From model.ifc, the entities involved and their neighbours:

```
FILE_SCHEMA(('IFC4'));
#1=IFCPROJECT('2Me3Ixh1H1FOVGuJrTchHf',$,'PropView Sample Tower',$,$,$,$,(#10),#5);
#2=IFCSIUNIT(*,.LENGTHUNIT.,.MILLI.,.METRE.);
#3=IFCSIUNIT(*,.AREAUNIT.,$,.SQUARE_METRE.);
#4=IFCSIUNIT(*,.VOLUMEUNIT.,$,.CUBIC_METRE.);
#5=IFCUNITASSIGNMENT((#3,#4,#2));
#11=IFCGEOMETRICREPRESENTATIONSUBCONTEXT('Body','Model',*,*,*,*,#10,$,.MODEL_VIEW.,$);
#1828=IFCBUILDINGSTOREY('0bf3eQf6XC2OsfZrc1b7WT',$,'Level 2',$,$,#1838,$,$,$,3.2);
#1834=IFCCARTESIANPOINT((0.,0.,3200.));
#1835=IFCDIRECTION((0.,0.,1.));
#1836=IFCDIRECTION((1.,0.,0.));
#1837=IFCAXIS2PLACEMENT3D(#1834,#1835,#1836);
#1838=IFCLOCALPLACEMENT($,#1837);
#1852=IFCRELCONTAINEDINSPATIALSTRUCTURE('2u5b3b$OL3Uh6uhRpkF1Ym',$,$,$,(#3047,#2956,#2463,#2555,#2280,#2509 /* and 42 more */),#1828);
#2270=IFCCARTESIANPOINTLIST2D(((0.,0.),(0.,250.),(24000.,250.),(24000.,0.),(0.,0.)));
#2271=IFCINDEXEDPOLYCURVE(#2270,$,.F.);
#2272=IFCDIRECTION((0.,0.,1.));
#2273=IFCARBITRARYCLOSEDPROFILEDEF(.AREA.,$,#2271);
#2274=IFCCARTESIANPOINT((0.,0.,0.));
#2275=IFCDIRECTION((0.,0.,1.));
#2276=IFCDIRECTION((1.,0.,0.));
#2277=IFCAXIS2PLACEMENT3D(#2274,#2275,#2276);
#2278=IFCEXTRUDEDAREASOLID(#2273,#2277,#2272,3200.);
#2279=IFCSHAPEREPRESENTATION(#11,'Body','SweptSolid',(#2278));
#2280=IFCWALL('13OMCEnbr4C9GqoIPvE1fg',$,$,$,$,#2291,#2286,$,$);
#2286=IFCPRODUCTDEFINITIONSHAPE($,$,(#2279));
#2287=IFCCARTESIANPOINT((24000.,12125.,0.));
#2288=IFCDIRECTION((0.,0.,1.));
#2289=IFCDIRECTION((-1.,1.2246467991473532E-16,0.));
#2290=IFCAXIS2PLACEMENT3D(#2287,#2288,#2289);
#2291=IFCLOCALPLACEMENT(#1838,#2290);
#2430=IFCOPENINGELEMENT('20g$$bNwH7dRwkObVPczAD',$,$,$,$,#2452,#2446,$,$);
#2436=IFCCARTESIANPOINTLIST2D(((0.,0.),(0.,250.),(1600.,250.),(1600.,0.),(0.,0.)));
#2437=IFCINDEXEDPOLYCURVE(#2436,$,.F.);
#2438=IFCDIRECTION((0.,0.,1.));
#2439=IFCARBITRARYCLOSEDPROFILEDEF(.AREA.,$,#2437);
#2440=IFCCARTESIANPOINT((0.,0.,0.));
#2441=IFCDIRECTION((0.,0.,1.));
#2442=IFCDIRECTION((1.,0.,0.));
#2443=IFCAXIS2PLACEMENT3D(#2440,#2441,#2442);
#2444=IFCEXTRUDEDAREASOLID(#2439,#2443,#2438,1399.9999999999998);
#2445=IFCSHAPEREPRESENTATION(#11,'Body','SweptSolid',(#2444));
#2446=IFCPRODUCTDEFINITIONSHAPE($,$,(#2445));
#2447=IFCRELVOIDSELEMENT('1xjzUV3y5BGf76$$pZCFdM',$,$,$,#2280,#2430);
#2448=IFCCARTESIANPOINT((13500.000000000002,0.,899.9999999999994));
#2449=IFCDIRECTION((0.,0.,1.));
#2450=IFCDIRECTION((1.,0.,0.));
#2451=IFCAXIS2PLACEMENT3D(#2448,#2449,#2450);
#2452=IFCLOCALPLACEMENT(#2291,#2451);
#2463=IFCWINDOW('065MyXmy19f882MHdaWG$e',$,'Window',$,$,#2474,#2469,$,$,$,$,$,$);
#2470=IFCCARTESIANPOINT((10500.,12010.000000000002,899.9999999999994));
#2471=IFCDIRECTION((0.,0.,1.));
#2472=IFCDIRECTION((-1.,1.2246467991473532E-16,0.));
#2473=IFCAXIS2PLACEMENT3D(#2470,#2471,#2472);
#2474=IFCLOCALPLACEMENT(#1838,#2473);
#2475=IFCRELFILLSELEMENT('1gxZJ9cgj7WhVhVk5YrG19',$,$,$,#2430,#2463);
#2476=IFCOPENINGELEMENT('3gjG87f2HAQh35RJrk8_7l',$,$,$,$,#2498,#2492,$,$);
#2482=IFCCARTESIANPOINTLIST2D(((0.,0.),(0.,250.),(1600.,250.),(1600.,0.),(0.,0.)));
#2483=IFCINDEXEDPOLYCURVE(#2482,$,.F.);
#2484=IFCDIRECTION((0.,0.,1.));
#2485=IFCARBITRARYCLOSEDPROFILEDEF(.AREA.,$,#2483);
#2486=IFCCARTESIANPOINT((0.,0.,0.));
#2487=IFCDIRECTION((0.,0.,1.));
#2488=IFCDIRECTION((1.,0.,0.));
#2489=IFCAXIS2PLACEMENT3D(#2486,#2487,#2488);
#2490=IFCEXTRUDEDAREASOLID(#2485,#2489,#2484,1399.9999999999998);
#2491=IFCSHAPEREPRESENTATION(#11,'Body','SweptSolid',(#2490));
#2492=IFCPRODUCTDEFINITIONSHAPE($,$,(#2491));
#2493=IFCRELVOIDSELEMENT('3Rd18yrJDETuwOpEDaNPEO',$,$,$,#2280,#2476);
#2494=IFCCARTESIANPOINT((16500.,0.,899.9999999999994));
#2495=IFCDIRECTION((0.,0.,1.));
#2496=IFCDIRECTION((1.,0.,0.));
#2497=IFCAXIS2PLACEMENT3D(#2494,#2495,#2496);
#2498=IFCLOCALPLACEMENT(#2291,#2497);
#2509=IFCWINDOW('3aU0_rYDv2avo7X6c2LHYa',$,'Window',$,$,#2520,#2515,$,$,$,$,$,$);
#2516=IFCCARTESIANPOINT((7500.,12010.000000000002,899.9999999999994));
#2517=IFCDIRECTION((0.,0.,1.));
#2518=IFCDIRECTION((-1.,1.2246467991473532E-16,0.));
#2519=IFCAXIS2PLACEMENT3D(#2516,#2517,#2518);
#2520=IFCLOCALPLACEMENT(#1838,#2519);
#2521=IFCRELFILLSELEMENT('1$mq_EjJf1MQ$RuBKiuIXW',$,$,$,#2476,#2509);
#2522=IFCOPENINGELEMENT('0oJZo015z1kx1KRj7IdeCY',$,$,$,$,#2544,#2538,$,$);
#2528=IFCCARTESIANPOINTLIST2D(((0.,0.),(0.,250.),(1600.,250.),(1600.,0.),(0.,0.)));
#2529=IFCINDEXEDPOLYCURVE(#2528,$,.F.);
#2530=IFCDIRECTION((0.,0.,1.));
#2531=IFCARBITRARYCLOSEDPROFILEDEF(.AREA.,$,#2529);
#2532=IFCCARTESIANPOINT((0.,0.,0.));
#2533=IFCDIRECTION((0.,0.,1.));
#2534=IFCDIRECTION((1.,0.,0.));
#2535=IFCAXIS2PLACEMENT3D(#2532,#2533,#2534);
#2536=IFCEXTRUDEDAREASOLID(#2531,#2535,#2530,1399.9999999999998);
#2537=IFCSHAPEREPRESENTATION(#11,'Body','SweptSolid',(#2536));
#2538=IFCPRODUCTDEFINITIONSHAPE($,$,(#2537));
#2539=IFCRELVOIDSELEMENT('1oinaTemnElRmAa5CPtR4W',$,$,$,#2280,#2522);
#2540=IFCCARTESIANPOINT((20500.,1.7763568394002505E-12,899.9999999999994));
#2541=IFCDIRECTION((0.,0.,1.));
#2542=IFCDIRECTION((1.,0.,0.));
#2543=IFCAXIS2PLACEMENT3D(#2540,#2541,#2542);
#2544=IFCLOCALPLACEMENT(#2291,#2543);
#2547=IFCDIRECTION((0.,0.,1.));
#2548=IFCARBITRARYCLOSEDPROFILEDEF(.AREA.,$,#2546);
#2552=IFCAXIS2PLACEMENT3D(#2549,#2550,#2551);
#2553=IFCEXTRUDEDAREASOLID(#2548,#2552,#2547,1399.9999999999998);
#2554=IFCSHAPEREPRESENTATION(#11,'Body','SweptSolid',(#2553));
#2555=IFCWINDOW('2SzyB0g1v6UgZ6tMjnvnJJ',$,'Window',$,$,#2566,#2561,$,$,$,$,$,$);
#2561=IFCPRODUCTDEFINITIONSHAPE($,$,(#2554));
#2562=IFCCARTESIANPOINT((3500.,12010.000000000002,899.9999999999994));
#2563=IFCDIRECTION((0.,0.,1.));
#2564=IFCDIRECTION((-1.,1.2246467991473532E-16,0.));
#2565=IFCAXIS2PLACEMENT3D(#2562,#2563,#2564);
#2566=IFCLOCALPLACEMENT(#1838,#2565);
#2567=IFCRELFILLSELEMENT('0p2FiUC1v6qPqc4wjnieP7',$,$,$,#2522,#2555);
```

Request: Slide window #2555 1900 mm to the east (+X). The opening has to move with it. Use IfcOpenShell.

```python
import ifcopenshell
import ifcopenshell.api.geometry
import ifcopenshell.util.placement
import ifcopenshell.util.unit

model = ifcopenshell.open("model.ifc")
unit_scale = ifcopenshell.util.unit.calculate_unit_scale(model)

window = model.by_id(2555)
opening = window.FillsVoids[0].RelatingOpeningElement
wall = opening.VoidsElements[0].RelatingBuildingElement

wall_matrix = ifcopenshell.util.placement.get_local_placement(wall.ObjectPlacement)
shift = wall_matrix[:3, 0] * -1.9 / unit_scale
before = ifcopenshell.util.placement.get_local_placement(window.ObjectPlacement)[:3, 3].copy()

# The window is not placed relative to its opening, so move both.
for product in (opening, window):
    matrix = ifcopenshell.util.placement.get_local_placement(product.ObjectPlacement)
    matrix[:3, 3] += shift
    ifcopenshell.api.geometry.edit_object_placement(model, product=product, matrix=matrix, is_si=False)

after = ifcopenshell.util.placement.get_local_placement(window.ObjectPlacement)[:3, 3]
print("window moved by", (after - before).round(3) + 0.0)

model.write("model-out.ifc")
```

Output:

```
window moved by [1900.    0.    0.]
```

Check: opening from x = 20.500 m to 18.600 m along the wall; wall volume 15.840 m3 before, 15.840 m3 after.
